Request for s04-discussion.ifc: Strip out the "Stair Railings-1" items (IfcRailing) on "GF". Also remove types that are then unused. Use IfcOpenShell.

First a look at what the model holds.

```python
import ifcopenshell
import ifcopenshell.util.element

model = ifcopenshell.open("s04-discussion.ifc")
print(model.schema)
storey = next(s for s in model.by_type("IfcBuildingStorey") if s.Name == "GF")
railings = [e for e in ifcopenshell.util.element.get_decomposition(storey) if e.is_a("IfcRailing")]
seen = {}
for e in railings:
    element_type = ifcopenshell.util.element.get_type(e)
    name = element_type.Name if element_type not in (None, e) else None
    seen[name] = seen.get(name, 0) + 1
for name, count in sorted(seen.items(), key=str):
    print(count, "x", name)
```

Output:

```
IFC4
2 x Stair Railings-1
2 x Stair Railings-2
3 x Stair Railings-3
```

```python
import ifcopenshell
import ifcopenshell.api.root
import ifcopenshell.util.element

model = ifcopenshell.open("s04-discussion.ifc")

storey = next(s for s in model.by_type("IfcBuildingStorey") if s.Name == "GF")
railings = [e for e in ifcopenshell.util.element.get_decomposition(storey) if e.is_a("IfcRailing")]
targets = [e for e in railings if (t := ifcopenshell.util.element.get_type(e)) not in (None, e) and t.Name == "Stair Railings-1"]
types = {ifcopenshell.util.element.get_type(e) for e in targets} - {None, *targets}

for e in targets:
    ifcopenshell.api.root.remove_product(model, product=e)
print(len(targets), "removed")

unused = [t for t in types if not ifcopenshell.util.element.get_types(t)]
for t in unused:
    ifcopenshell.api.root.remove_product(model, product=t)
print(len(unused), "unused types removed")

model.write("s04-discussion_edited.ifc")
```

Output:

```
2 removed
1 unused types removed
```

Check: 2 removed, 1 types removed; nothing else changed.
